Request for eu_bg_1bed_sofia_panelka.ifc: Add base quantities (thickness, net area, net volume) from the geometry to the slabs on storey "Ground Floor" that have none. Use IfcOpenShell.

First a look at what the model holds.

```python
import ifcopenshell
import ifcopenshell.util.element
import ifcopenshell.util.unit

model = ifcopenshell.open("eu_bg_1bed_sofia_panelka.ifc")
print(model.schema)
for unit_type in ("LENGTHUNIT", "AREAUNIT", "VOLUMEUNIT"):
    print(unit_type, ifcopenshell.util.unit.calculate_unit_scale(model, unit_type))
storey = next(s for s in model.by_type("IfcBuildingStorey") if s.Name == "Ground Floor")
slabs = [e for e in ifcopenshell.util.element.get_decomposition(storey) if e.is_a("IfcSlab")]
for e in sorted(slabs, key=lambda e: e.id()):
    print(e.id(), e.is_a(), e.Name, list(ifcopenshell.util.element.get_psets(e, qtos_only=True)), sep=" | ")
```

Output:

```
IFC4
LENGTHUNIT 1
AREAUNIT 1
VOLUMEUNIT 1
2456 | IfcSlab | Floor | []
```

```python
import ifcopenshell
import ifcopenshell.api.pset
import ifcopenshell.geom
import ifcopenshell.util.element
import ifcopenshell.util.shape
import ifcopenshell.util.unit

model = ifcopenshell.open("eu_bg_1bed_sofia_panelka.ifc")
unit_scale = ifcopenshell.util.unit.calculate_unit_scale(model)
area_scale = ifcopenshell.util.unit.calculate_unit_scale(model, "AREAUNIT")
volume_scale = ifcopenshell.util.unit.calculate_unit_scale(model, "VOLUMEUNIT")
settings = ifcopenshell.geom.settings()

storey = next(s for s in model.by_type("IfcBuildingStorey") if s.Name == "Ground Floor")
slabs = [e for e in ifcopenshell.util.element.get_decomposition(storey) if e.is_a("IfcSlab")]

for e in sorted(slabs, key=lambda e: e.id()):
    if ifcopenshell.util.element.get_psets(e, qtos_only=True, should_inherit=False):
        continue
    # Geometry comes back in metres, in the element's own axes.
    shape = ifcopenshell.geom.create_shape(settings, e)
    values = {
        "Width": ifcopenshell.util.shape.get_z(shape.geometry) / unit_scale,
        "NetArea": ifcopenshell.util.shape.get_footprint_area(shape.geometry) / area_scale,
        "NetVolume": ifcopenshell.util.shape.get_volume(shape.geometry) / volume_scale,
    }
    qto = ifcopenshell.api.pset.add_qto(model, product=e, name="Qto_SlabBaseQuantities")
    ifcopenshell.api.pset.edit_qto(model, qto=qto, properties=values)
    print(e.id(), {k: round(v, 3) for k, v in values.items()})

model.write("eu_bg_1bed_sofia_panelka_v2.ifc")
```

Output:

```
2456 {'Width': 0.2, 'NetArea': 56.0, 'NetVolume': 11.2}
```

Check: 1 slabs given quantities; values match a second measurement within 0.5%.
